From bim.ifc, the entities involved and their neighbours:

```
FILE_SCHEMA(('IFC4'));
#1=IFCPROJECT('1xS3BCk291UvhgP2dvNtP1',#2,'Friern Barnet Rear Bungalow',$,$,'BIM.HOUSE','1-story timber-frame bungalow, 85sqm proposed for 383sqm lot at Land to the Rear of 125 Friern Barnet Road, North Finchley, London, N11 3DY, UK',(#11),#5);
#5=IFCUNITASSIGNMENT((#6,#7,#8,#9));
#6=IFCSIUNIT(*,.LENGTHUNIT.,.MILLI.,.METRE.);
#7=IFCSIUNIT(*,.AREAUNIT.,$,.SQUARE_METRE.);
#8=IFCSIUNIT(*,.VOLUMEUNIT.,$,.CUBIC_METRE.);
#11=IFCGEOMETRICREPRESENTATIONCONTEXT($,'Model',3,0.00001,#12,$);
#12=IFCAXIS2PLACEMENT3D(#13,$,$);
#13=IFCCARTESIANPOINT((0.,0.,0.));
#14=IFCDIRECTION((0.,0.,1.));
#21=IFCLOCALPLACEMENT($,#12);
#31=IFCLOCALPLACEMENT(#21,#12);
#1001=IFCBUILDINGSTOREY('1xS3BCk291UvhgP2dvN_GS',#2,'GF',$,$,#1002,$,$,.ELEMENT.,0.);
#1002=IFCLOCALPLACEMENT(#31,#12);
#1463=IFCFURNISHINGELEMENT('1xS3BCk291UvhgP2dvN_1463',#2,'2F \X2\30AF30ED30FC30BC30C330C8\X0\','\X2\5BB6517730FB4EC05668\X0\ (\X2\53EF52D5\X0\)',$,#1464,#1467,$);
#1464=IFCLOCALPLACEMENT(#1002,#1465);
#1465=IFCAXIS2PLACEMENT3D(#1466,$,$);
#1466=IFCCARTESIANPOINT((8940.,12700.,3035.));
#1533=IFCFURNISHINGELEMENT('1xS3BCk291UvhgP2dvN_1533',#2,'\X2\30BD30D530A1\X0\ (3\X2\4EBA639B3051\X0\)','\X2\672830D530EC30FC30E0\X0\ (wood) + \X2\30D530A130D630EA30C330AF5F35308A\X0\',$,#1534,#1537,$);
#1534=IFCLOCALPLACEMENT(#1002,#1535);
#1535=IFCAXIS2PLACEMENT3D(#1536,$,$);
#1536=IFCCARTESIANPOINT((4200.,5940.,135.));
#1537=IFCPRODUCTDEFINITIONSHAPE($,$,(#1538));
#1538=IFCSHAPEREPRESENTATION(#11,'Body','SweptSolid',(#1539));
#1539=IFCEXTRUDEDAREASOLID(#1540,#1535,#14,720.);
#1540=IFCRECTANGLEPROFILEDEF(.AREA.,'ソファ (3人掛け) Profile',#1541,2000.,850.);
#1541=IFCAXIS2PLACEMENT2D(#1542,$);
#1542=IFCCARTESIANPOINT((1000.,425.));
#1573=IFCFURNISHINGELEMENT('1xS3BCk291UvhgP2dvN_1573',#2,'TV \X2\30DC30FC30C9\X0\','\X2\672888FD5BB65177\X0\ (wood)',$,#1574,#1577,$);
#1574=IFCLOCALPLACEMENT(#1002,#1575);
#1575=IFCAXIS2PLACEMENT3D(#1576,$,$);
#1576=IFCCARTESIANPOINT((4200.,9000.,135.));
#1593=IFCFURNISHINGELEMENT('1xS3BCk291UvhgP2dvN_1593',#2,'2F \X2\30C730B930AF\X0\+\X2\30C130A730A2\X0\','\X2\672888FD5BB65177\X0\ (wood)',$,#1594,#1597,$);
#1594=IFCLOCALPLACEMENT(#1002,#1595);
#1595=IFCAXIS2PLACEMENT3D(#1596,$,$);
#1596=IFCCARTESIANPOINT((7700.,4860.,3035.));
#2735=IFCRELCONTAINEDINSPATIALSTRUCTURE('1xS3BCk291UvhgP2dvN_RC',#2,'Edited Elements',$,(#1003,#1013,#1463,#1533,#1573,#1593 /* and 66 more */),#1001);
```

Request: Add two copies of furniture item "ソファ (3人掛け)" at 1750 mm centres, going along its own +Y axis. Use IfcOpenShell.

```python
import ifcopenshell
import ifcopenshell.api.geometry
import ifcopenshell.api.root
import ifcopenshell.util.element
import ifcopenshell.util.placement
import ifcopenshell.util.unit

model = ifcopenshell.open("bim.ifc")
unit_scale = ifcopenshell.util.unit.calculate_unit_scale(model)


def reuse_history(source, copy):
    """copy_class also copies each property set's owner history, people and application; keep the originals."""
    for rel in copy.IsDefinedBy:
        if rel.is_a("IfcRelDefinesByProperties") and (history := rel.RelatingPropertyDefinition.OwnerHistory):
            rel.RelatingPropertyDefinition.OwnerHistory = source.OwnerHistory
            ifcopenshell.util.element.remove_deep2(model, history)


source = model.by_guid("1xS3BCk291UvhgP2dvN_1533")
base = ifcopenshell.util.placement.get_local_placement(source.ObjectPlacement)
step = base[:3, 1] * 1.75 / unit_scale

for i in range(1, 3):
    copy = ifcopenshell.api.root.copy_class(model, product=source)
    copy.Representation = ifcopenshell.util.element.copy_deep(
        model, source.Representation, exclude=["IfcGeometricRepresentationContext", "IfcRepresentationMap"]
    )
    reuse_history(source, copy)
    matrix = base.copy()
    matrix[:3, 3] += i * step
    print("added at", matrix[:3, 3].round(3) + 0.0)
    ifcopenshell.api.geometry.edit_object_placement(model, product=copy, matrix=matrix, is_si=False)

model.write("bim_rev.ifc")
```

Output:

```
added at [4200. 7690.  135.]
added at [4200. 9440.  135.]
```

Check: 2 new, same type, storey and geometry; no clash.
